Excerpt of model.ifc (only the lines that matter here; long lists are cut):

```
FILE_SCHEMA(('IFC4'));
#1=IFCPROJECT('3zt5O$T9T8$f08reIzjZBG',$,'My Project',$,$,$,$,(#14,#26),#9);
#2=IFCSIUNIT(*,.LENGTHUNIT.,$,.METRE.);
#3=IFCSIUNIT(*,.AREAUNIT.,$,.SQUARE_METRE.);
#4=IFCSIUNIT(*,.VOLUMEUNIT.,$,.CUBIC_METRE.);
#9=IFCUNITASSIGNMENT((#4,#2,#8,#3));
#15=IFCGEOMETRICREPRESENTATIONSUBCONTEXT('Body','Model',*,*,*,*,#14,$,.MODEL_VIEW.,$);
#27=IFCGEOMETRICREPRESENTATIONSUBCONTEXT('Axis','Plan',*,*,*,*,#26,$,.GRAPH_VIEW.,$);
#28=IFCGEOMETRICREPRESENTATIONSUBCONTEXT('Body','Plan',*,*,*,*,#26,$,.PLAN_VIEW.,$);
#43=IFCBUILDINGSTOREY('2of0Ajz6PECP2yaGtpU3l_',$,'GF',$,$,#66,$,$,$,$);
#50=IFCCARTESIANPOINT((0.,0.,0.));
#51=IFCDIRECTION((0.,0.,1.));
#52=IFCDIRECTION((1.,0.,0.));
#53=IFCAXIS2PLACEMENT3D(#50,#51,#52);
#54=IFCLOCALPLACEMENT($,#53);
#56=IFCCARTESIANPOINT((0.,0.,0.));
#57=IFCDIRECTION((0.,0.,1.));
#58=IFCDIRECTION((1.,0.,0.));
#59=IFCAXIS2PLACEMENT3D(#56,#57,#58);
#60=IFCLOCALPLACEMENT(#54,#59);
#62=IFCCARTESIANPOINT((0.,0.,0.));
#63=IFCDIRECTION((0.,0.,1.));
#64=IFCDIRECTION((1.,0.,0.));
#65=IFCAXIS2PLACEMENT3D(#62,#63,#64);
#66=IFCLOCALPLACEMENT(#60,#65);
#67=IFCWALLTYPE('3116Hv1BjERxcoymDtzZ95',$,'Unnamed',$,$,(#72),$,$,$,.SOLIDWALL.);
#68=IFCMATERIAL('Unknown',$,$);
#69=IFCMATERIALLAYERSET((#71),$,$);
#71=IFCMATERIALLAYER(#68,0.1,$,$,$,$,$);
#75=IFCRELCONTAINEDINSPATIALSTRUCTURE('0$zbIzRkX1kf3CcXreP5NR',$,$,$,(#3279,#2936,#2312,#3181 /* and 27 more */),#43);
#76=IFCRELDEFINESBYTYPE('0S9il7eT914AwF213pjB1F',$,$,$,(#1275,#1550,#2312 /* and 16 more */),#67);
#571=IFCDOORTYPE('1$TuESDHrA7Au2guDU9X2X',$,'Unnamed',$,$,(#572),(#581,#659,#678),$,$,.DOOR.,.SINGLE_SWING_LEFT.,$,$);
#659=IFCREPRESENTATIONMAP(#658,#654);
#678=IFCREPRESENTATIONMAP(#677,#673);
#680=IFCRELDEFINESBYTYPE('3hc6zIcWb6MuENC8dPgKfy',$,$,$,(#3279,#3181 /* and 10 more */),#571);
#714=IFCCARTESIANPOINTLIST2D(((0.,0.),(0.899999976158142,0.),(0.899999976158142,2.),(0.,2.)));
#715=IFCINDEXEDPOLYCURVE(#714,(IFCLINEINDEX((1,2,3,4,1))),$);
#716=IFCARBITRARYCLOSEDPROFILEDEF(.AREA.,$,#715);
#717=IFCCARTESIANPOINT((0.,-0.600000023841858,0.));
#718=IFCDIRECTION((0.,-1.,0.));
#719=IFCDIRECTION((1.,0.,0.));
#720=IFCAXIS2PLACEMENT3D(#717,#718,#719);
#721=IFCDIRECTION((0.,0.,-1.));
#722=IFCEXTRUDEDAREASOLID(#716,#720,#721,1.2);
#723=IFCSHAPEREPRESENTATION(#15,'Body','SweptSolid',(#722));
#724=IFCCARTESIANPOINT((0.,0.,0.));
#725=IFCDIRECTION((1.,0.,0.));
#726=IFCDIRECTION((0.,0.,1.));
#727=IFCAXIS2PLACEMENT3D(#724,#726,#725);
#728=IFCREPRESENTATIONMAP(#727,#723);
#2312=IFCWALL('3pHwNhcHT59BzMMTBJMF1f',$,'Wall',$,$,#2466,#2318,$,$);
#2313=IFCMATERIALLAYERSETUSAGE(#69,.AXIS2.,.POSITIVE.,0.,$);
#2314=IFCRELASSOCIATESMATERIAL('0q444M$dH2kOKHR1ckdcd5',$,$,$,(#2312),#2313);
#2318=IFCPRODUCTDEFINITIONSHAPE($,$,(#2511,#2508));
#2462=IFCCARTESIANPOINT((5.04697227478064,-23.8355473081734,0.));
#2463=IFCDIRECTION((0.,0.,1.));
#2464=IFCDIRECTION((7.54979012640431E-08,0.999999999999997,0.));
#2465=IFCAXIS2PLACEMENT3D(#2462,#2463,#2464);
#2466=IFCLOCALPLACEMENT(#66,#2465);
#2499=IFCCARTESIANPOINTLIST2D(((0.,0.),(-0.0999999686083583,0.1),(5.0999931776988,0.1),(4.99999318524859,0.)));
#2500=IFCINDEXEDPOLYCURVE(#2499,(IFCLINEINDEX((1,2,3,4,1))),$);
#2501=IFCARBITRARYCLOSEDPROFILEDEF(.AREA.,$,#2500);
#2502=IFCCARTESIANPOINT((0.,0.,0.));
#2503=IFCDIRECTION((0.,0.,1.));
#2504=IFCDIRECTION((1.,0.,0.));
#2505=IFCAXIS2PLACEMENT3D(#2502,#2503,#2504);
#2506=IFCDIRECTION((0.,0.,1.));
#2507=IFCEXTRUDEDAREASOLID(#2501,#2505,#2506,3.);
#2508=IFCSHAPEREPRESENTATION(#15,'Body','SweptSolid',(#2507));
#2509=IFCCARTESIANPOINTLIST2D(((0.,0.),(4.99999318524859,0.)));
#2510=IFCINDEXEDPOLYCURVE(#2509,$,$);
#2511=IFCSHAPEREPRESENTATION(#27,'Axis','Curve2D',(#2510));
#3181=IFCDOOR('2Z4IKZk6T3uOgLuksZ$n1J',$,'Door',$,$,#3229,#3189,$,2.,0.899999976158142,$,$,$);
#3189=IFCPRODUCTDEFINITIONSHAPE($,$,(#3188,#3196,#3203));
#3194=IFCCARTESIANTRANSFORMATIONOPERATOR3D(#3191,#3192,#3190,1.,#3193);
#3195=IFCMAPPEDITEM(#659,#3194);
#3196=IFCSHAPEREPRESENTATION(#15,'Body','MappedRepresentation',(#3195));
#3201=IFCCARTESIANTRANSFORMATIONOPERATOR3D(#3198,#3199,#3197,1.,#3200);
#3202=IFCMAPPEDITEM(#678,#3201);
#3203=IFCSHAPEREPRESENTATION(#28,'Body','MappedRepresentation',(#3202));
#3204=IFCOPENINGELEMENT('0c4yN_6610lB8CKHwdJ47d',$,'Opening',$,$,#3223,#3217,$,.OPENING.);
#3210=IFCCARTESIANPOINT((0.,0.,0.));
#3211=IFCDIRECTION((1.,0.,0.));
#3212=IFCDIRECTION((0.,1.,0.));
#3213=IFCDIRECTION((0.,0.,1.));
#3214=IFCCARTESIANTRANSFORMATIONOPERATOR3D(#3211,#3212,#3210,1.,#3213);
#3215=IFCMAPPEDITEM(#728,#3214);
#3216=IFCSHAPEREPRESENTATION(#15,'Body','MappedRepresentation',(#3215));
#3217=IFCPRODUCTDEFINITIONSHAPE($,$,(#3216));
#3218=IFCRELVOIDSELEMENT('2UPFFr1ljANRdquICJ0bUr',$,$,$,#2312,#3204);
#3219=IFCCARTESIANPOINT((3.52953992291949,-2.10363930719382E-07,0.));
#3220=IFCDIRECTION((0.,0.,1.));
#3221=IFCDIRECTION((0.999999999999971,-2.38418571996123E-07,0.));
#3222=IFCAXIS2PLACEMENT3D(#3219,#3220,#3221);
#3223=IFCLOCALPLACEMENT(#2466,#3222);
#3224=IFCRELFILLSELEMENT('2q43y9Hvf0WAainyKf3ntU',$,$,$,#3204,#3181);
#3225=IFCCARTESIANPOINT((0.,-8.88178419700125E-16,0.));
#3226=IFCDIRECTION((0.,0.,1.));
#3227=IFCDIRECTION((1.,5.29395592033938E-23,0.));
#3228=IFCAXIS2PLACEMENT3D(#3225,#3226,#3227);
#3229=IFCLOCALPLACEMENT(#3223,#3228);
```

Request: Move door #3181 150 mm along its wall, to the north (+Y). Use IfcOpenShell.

```python
import ifcopenshell
import ifcopenshell.api.geometry
import ifcopenshell.util.placement

model = ifcopenshell.open("model.ifc")

door = model.by_id(3181)
opening = door.FillsVoids[0].RelatingOpeningElement
wall = opening.VoidsElements[0].RelatingBuildingElement

wall_matrix = ifcopenshell.util.placement.get_local_placement(wall.ObjectPlacement)
shift = wall_matrix[:3, 0] * 0.15
before = ifcopenshell.util.placement.get_local_placement(door.ObjectPlacement)[:3, 3].copy()

# The door is placed relative to its opening, so it follows when the opening moves.
matrix = ifcopenshell.util.placement.get_local_placement(opening.ObjectPlacement)
matrix[:3, 3] += shift
ifcopenshell.api.geometry.edit_object_placement(
    model, product=opening, matrix=matrix, is_si=False, should_transform_children=True
)

after = ifcopenshell.util.placement.get_local_placement(door.ObjectPlacement)[:3, 3]
print("door moved by", (after - before).round(3) + 0.0)

model.write("model_edited.ifc")
```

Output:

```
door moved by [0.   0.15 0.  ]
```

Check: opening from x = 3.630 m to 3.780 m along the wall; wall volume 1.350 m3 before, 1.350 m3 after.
